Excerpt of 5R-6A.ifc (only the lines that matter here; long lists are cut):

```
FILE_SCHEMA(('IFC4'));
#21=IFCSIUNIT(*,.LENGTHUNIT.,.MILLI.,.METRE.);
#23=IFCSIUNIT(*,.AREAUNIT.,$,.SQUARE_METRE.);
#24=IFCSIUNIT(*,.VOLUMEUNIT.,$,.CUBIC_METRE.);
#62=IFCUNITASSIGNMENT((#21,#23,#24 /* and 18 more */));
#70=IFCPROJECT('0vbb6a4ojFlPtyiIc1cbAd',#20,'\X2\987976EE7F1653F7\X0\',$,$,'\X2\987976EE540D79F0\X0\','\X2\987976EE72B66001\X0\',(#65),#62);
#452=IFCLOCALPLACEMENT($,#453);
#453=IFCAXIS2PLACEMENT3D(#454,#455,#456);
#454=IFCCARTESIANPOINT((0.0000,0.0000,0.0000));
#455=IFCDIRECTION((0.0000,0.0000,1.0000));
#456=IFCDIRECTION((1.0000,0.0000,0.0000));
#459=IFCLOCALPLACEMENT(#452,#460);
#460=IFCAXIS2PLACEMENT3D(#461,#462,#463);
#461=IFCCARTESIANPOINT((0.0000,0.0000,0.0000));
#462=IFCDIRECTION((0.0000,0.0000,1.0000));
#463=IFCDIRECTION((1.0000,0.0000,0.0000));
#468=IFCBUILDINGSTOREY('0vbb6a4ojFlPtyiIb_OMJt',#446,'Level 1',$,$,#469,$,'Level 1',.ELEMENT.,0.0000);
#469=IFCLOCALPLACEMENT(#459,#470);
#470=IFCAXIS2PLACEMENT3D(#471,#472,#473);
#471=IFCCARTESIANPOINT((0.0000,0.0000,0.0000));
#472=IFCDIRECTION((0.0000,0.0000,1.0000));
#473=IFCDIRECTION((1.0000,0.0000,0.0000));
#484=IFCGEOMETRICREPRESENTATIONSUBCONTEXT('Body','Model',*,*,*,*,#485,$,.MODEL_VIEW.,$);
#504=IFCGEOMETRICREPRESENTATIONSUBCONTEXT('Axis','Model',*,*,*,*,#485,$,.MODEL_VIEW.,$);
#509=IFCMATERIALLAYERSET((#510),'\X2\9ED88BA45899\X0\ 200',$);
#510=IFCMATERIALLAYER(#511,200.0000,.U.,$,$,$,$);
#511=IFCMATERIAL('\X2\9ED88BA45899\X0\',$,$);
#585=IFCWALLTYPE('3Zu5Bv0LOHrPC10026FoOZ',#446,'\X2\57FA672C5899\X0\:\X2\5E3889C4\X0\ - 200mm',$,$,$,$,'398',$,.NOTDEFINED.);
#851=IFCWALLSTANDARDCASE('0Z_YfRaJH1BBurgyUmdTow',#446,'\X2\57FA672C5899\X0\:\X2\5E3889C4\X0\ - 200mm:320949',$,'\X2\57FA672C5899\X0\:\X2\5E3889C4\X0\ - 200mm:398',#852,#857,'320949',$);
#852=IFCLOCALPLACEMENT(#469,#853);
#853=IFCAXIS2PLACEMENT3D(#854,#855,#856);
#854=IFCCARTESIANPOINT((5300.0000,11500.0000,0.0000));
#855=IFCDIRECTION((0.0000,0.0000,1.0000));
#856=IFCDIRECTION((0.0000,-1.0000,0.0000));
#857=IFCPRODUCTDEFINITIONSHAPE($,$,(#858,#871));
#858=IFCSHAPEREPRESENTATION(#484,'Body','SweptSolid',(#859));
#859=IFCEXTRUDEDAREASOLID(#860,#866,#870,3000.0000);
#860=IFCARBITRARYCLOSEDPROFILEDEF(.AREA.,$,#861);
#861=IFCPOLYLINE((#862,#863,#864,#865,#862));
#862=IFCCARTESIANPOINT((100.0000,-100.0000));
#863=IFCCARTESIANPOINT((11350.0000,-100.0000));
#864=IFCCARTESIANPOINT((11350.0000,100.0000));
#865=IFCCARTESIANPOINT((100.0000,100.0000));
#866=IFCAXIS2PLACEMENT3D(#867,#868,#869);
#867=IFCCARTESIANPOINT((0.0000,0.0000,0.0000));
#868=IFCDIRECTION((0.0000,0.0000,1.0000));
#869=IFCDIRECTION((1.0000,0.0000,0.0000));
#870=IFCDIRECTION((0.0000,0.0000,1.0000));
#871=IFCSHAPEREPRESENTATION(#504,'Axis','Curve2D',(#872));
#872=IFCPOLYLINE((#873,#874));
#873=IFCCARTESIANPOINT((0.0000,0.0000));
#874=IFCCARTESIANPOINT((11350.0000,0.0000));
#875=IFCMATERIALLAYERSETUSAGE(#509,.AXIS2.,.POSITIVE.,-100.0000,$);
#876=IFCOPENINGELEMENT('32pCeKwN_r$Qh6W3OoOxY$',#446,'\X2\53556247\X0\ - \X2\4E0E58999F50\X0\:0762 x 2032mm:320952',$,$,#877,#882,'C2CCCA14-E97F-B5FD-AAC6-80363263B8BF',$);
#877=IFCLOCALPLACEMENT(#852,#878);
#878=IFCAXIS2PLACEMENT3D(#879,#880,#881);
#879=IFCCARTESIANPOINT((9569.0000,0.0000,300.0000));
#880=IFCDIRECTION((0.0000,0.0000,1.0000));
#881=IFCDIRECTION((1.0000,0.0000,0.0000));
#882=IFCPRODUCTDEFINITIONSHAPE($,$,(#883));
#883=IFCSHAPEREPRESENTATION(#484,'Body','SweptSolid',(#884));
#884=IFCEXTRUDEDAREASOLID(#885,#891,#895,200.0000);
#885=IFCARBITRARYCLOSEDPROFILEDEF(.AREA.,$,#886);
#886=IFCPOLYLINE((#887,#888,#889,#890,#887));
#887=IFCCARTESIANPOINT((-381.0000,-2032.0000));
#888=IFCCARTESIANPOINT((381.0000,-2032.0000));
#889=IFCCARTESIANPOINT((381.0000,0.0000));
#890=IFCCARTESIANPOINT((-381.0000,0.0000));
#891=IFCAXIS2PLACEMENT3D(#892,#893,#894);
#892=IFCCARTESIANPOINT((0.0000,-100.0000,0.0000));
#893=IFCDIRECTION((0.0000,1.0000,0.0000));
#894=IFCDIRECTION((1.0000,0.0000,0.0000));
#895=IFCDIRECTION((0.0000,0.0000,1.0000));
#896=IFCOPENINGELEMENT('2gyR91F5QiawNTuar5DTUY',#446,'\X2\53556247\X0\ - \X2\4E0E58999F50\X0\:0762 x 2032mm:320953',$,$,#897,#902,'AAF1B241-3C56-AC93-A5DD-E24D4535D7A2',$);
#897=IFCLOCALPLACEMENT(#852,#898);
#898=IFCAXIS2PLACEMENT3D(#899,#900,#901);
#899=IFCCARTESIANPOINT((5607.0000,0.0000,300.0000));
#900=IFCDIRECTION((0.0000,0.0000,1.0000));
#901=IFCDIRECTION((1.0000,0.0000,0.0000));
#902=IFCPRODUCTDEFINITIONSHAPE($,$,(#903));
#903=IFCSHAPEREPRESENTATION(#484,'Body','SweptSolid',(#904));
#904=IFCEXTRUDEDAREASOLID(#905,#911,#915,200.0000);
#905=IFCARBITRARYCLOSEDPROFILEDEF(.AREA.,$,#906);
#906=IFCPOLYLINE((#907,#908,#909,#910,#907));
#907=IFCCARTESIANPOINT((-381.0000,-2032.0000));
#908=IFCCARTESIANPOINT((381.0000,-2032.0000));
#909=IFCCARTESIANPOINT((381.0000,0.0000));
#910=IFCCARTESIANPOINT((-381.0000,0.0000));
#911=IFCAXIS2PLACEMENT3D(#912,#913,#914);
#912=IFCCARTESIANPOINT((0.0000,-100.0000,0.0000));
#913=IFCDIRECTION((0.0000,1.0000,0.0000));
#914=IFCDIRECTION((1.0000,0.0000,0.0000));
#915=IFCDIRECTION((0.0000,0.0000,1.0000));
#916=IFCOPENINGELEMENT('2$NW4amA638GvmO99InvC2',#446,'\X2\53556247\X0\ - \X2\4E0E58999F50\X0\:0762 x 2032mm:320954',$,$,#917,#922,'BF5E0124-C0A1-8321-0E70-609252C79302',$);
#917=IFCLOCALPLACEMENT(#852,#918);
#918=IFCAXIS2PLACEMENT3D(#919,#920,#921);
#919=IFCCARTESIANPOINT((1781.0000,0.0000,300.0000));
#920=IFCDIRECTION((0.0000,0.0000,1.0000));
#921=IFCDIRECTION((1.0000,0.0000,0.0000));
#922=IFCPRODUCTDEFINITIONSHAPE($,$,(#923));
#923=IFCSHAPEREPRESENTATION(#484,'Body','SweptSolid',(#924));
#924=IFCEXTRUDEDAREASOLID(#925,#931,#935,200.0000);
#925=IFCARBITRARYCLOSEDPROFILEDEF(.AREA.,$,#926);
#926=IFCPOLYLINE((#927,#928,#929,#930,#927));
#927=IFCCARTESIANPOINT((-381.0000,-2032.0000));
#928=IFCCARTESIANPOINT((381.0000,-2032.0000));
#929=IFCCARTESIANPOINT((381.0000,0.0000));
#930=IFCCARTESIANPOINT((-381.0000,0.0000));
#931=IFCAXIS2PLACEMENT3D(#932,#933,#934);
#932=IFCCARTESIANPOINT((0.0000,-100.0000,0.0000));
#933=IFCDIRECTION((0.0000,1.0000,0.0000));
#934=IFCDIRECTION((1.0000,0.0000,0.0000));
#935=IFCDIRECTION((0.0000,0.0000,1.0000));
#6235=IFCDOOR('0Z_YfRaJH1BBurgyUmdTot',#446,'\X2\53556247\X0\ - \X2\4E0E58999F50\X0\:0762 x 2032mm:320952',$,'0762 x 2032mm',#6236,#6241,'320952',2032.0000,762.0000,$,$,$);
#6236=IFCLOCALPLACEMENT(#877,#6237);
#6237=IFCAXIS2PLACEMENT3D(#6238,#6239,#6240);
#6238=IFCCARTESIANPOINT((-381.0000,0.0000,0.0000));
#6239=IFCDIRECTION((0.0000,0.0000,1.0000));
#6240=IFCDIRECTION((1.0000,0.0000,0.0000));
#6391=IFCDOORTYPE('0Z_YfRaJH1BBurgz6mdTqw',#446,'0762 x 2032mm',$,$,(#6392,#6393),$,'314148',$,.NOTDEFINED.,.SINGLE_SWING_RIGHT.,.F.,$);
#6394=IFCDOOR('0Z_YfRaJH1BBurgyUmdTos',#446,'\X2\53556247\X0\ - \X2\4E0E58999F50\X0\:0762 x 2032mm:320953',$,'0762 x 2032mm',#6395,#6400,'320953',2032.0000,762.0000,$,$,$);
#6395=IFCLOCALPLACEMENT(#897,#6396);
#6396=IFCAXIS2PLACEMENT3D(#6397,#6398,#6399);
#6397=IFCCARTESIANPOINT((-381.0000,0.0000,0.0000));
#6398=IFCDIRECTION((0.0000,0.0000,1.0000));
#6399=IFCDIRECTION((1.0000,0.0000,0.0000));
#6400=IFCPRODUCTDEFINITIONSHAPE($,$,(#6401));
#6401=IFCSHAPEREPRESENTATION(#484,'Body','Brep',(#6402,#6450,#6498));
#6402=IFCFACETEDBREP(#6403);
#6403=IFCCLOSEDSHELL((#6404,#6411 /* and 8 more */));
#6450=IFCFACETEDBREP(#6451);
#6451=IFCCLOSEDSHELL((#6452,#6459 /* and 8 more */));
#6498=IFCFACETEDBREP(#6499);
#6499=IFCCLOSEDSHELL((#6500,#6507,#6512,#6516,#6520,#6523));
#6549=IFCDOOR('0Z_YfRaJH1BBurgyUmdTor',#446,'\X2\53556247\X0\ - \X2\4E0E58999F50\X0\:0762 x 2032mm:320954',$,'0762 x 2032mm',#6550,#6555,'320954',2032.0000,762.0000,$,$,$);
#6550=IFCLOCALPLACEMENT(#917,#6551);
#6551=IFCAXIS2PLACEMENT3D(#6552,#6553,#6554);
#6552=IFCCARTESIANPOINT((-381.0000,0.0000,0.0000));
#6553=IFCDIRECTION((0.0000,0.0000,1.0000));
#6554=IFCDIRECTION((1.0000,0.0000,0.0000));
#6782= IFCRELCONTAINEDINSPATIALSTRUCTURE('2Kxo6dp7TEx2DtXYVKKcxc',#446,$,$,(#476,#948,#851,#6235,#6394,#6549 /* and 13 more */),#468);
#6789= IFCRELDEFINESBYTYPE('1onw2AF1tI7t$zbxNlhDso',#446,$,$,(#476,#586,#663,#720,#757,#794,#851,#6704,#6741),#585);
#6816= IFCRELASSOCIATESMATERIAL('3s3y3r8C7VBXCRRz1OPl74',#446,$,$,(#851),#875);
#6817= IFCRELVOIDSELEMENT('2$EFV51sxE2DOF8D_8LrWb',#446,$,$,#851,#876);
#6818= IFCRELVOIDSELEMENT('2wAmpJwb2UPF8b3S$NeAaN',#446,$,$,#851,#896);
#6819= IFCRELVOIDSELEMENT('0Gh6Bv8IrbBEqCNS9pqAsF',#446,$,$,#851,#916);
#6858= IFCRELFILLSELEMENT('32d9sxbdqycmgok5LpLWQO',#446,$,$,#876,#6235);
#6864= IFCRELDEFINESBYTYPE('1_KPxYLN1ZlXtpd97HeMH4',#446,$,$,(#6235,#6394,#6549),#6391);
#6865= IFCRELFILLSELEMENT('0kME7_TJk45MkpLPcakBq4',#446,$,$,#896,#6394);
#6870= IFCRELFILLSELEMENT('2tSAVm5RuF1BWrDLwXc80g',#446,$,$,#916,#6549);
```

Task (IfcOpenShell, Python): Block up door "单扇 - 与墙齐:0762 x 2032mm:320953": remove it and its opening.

```python
import ifcopenshell
import ifcopenshell.api.feature
import ifcopenshell.api.root
import ifcopenshell.geom
import ifcopenshell.util.shape

model = ifcopenshell.open("5R-6A.ifc")
settings = ifcopenshell.geom.settings()


def volume(element):
    """Net volume in cubic metres, openings subtracted."""
    shape = ifcopenshell.geom.create_shape(settings, element)
    return ifcopenshell.util.shape.get_volume(shape.geometry)


door = model.by_guid("0Z_YfRaJH1BBurgyUmdTos")
opening = door.FillsVoids[0].RelatingOpeningElement
wall = opening.VoidsElements[0].RelatingBuildingElement
before = volume(wall)

ifcopenshell.api.root.remove_product(model, product=door)
ifcopenshell.api.feature.remove_feature(model, feature=opening)

after = volume(wall)

print(f"wall volume {before:.3f} -> {after:.3f} m3")

model.write("5R-6A-out.ifc")
```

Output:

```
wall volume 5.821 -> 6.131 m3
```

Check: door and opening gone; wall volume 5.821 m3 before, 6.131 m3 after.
